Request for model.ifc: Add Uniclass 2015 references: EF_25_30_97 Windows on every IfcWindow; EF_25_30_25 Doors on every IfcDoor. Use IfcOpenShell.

First a look at what the model holds.

```python
import ifcopenshell

model = ifcopenshell.open("model.ifc")
print(model.schema)
print("classifications:", [c.Name for c in model.by_type("IfcClassification")])
for ifc_class in ("IfcDoor", "IfcRoof", "IfcStair", "IfcWall", "IfcWindow"):
    print(ifc_class, len(model.by_type(ifc_class)))
```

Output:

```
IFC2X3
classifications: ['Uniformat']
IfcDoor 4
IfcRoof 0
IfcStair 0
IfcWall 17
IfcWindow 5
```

```python
import ifcopenshell
import ifcopenshell.api.classification

model = ifcopenshell.open("model.ifc")

# IFC2X3 requires Source and Edition and has no link from the project to the system.
system = model.create_entity("IfcClassification", Source="NBS", Edition="2015", Name="Uniclass 2015")

codes = {
    "IfcWindow": ("EF_25_30_97", "Windows"),
    "IfcDoor": ("EF_25_30_25", "Doors"),
}
for ifc_class, (code, name) in codes.items():
    products = model.by_type(ifc_class)
    ifcopenshell.api.classification.add_reference(
        model, products=products, classification=system, identification=code, name=name
    )
    print(code, len(products))

model.write("model_v2.ifc")
```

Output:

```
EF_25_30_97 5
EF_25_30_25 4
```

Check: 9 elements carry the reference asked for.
